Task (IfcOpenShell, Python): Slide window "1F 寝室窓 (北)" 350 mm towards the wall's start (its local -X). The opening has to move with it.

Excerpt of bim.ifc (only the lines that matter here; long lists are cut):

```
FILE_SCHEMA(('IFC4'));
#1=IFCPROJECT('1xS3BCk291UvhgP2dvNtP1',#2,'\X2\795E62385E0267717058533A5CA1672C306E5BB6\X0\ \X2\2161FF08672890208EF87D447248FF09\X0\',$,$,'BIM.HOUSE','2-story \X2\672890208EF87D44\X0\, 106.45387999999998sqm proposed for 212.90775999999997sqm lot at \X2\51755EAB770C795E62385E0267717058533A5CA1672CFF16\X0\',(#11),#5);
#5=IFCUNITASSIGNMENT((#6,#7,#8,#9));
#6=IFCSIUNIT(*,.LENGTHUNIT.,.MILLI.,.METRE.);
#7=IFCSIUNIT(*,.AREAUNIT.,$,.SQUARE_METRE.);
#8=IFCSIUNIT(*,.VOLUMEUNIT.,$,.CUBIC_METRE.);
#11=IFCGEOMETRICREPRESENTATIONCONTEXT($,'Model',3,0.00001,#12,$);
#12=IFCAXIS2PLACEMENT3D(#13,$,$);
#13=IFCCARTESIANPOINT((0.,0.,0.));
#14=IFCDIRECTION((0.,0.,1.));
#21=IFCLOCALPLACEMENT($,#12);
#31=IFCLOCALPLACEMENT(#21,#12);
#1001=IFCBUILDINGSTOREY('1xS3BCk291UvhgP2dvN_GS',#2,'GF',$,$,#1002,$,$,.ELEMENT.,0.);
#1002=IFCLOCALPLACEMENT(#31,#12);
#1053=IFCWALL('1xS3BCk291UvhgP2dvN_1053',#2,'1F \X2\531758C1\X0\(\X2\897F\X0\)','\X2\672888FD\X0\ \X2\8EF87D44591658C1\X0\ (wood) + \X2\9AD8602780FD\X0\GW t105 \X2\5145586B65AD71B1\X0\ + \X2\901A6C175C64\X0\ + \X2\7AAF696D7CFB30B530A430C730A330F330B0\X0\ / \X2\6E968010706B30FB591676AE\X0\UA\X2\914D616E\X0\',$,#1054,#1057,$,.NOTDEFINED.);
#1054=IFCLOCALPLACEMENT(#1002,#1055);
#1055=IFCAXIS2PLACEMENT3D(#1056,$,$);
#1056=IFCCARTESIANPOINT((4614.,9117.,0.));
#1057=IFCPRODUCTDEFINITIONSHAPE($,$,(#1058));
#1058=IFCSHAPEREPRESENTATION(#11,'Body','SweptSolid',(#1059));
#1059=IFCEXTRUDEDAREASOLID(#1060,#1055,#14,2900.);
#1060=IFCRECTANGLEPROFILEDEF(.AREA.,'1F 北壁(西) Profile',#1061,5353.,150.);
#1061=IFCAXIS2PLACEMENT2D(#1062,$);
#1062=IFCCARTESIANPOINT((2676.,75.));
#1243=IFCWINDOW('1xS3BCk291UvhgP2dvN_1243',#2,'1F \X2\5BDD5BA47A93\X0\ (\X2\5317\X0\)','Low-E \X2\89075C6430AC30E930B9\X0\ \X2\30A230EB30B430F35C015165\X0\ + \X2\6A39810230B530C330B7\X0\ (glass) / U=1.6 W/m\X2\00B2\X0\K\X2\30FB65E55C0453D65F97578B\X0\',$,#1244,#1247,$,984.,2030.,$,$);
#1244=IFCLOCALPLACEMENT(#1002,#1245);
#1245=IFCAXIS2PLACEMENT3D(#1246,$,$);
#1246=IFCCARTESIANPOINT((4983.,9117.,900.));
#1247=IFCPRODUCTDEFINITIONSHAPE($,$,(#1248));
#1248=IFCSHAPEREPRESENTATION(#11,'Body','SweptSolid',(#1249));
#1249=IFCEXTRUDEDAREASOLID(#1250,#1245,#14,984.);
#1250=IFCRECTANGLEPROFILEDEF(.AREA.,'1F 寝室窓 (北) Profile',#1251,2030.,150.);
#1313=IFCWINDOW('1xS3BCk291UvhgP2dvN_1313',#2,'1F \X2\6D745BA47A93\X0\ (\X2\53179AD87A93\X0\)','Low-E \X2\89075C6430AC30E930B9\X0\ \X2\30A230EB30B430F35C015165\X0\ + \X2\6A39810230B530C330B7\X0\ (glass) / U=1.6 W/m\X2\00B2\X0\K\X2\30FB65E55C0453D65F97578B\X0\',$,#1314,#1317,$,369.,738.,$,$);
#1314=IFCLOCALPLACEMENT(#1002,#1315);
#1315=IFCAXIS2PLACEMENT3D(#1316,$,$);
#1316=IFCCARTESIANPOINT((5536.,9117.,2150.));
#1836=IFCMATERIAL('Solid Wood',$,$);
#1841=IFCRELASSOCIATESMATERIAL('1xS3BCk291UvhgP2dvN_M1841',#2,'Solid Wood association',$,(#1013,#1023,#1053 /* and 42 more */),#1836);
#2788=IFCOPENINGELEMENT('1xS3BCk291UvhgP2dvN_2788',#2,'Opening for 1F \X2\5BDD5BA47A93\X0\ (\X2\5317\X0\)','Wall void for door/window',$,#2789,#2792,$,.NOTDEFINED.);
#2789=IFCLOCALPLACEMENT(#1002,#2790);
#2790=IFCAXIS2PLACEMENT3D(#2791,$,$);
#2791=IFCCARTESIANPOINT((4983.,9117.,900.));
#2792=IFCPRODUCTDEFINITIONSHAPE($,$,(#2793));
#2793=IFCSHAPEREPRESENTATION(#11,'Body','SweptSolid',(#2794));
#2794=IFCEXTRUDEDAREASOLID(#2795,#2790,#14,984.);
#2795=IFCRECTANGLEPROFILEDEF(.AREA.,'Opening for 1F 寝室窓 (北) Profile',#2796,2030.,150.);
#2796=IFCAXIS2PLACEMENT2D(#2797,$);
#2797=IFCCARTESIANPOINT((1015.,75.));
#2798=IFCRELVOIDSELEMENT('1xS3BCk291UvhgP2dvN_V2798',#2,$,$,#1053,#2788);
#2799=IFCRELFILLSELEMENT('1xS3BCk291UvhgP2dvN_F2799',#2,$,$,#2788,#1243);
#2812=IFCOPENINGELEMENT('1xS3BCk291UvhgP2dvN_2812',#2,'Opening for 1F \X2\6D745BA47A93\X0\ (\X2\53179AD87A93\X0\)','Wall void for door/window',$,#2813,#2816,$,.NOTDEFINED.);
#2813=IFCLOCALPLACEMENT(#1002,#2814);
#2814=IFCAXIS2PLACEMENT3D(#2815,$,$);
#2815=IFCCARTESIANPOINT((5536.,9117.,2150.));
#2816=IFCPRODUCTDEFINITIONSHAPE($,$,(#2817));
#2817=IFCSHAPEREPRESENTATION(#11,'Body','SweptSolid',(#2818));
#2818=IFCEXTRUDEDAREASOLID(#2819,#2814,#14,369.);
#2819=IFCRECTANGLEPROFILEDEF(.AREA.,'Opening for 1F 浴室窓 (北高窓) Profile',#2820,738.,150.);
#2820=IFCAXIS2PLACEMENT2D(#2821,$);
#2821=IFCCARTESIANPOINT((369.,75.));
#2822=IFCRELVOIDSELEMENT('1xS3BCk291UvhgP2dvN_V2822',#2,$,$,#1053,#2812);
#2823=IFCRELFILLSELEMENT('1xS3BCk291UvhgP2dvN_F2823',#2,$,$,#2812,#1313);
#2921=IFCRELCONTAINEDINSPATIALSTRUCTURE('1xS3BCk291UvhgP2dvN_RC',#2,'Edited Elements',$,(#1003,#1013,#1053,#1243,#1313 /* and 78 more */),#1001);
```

```python
import ifcopenshell
import ifcopenshell.api.geometry
import ifcopenshell.util.placement

model = ifcopenshell.open("bim.ifc")

window = model.by_id(1243)
opening = window.FillsVoids[0].RelatingOpeningElement
wall = opening.VoidsElements[0].RelatingBuildingElement

wall_matrix = ifcopenshell.util.placement.get_local_placement(wall.ObjectPlacement)
shift = wall_matrix[:3, 0] * -350.0
before = ifcopenshell.util.placement.get_local_placement(window.ObjectPlacement)[:3, 3].copy()

# The window is not placed relative to its opening, so move both.
for product in (opening, window):
    matrix = ifcopenshell.util.placement.get_local_placement(product.ObjectPlacement)
    matrix[:3, 3] += shift
    ifcopenshell.api.geometry.edit_object_placement(model, product=product, matrix=matrix, is_si=False)

after = ifcopenshell.util.placement.get_local_placement(window.ObjectPlacement)[:3, 3]
print("window moved by", (after - before).round(3) + 0.0)

model.write("bim_edited.ifc")
```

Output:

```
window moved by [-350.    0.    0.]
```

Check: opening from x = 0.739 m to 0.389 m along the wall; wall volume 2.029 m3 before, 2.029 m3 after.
